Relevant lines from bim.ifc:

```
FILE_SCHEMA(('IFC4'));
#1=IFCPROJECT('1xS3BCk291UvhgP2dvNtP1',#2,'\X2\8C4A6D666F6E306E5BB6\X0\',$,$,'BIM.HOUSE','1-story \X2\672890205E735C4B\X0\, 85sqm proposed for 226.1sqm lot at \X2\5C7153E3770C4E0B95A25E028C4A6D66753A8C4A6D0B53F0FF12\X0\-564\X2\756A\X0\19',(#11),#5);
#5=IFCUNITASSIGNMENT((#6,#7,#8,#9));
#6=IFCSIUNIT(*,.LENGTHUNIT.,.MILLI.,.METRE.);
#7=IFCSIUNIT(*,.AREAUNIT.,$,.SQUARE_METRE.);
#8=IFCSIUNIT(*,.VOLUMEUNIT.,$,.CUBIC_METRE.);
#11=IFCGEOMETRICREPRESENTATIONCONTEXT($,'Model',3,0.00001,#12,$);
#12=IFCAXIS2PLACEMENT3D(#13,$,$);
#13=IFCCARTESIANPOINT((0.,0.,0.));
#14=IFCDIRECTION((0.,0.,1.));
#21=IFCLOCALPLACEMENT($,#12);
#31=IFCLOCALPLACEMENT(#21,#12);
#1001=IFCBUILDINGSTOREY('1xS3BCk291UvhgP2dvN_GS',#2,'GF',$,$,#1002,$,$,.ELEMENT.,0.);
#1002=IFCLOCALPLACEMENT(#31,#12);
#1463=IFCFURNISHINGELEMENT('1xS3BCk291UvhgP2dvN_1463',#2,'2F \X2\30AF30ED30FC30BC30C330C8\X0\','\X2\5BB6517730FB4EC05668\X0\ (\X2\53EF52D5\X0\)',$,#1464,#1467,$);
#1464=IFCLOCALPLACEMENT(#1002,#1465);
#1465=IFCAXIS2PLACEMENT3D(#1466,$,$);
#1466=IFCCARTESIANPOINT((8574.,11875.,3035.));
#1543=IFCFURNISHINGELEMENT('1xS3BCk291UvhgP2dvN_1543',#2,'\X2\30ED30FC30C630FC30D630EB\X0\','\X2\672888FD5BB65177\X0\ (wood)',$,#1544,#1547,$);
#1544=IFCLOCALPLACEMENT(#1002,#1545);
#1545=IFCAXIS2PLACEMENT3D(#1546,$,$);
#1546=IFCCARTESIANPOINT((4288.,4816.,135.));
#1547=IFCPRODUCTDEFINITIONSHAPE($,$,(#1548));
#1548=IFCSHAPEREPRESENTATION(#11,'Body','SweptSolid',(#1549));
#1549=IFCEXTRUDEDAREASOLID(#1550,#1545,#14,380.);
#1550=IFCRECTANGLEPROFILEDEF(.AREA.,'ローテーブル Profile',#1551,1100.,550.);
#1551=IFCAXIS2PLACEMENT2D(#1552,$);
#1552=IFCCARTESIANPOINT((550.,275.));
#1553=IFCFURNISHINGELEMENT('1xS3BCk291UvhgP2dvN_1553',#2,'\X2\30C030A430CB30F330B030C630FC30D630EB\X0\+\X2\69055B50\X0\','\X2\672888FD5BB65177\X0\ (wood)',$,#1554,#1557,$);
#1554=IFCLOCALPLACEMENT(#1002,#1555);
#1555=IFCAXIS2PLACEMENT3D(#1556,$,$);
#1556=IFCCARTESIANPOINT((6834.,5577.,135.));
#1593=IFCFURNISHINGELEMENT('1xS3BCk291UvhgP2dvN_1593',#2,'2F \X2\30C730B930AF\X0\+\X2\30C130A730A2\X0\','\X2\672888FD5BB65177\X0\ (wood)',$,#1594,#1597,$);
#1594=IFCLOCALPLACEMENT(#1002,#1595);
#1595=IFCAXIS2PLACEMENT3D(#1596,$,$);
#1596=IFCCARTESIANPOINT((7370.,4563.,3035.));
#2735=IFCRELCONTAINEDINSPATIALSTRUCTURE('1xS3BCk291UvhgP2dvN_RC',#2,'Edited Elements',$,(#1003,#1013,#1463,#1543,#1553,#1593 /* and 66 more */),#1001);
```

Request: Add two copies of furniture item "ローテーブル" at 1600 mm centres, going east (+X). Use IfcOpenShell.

```python
import numpy as np
import ifcopenshell
import ifcopenshell.api.geometry
import ifcopenshell.api.root
import ifcopenshell.util.element
import ifcopenshell.util.placement
import ifcopenshell.util.unit

model = ifcopenshell.open("bim.ifc")
unit_scale = ifcopenshell.util.unit.calculate_unit_scale(model)


def reuse_history(source, copy):
    """copy_class also copies each property set's owner history, people and application; keep the originals."""
    for rel in copy.IsDefinedBy:
        if rel.is_a("IfcRelDefinesByProperties") and (history := rel.RelatingPropertyDefinition.OwnerHistory):
            rel.RelatingPropertyDefinition.OwnerHistory = source.OwnerHistory
            ifcopenshell.util.element.remove_deep2(model, history)


source = model.by_id(1543)
base = ifcopenshell.util.placement.get_local_placement(source.ObjectPlacement)
step = np.array([1.0, 0.0, 0.0]) * 1.6 / unit_scale

for i in range(1, 3):
    copy = ifcopenshell.api.root.copy_class(model, product=source)
    copy.Representation = ifcopenshell.util.element.copy_deep(
        model, source.Representation, exclude=["IfcGeometricRepresentationContext", "IfcRepresentationMap"]
    )
    reuse_history(source, copy)
    matrix = base.copy()
    matrix[:3, 3] += i * step
    print("added at", matrix[:3, 3].round(3) + 0.0)
    ifcopenshell.api.geometry.edit_object_placement(model, product=copy, matrix=matrix, is_si=False)

model.write("bim_v2.ifc")
```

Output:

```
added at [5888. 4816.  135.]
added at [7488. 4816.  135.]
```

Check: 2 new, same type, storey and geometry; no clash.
